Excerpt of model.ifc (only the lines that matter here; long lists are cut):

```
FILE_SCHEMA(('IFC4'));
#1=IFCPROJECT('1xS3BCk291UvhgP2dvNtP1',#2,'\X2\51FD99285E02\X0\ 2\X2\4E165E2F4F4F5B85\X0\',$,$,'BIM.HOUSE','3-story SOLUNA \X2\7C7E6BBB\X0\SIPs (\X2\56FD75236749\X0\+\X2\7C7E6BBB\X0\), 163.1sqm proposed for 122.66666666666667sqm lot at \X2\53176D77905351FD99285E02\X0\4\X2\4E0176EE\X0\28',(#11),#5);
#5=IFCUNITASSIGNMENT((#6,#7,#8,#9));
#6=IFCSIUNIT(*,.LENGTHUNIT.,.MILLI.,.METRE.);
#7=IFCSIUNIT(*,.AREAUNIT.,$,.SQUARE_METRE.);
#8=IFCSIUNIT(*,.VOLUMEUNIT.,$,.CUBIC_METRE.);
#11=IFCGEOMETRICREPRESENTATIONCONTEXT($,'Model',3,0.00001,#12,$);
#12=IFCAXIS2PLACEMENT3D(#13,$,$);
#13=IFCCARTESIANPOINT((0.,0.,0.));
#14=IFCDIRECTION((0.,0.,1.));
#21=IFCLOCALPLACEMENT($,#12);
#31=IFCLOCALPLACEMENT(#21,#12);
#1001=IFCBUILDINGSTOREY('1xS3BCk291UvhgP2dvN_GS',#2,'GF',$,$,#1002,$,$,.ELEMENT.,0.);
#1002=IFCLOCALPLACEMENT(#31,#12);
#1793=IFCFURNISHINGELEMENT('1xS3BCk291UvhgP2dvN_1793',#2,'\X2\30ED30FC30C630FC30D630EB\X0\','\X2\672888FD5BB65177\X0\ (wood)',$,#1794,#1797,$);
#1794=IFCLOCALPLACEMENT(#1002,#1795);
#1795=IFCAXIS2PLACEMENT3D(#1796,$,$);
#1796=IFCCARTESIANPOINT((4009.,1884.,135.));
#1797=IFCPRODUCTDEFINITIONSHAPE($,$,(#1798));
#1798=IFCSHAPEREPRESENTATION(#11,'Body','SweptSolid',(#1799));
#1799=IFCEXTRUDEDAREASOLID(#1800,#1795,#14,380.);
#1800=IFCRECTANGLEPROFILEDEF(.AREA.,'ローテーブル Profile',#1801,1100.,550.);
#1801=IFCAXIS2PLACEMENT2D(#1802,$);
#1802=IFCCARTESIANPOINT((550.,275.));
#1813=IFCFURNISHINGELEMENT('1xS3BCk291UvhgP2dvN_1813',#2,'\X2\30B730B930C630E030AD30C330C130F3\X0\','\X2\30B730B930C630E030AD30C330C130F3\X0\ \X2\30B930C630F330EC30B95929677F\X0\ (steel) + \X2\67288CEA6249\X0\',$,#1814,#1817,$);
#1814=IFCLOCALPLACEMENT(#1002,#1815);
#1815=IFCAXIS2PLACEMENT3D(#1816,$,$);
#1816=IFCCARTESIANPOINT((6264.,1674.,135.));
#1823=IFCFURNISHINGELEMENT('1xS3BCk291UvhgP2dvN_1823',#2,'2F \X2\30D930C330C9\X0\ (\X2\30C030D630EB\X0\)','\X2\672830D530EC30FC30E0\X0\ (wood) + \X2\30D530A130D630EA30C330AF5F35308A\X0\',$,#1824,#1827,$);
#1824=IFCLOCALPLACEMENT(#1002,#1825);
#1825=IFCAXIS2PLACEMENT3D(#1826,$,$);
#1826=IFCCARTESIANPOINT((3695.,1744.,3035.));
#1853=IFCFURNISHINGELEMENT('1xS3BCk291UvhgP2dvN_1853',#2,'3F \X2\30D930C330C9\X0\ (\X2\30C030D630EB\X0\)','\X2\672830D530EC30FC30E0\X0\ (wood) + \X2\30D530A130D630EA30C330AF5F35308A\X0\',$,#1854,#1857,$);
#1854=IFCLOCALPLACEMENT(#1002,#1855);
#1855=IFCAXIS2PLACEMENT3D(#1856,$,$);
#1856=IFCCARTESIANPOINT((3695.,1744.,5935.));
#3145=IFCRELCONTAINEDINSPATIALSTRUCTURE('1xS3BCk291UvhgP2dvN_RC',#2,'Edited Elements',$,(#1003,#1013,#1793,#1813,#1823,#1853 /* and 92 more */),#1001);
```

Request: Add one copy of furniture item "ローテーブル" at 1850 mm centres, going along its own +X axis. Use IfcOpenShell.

```python
import ifcopenshell
import ifcopenshell.api.geometry
import ifcopenshell.api.root
import ifcopenshell.util.element
import ifcopenshell.util.placement

model = ifcopenshell.open("model.ifc")


def reuse_history(source, copy):
    """copy_class also copies each property set's owner history, people and application; keep the originals."""
    for rel in copy.IsDefinedBy:
        if rel.is_a("IfcRelDefinesByProperties") and (history := rel.RelatingPropertyDefinition.OwnerHistory):
            rel.RelatingPropertyDefinition.OwnerHistory = source.OwnerHistory
            ifcopenshell.util.element.remove_deep2(model, history)


source = model.by_guid("1xS3BCk291UvhgP2dvN_1793")
base = ifcopenshell.util.placement.get_local_placement(source.ObjectPlacement)
step = base[:3, 0] * 1850.0

for i in range(1, 2):
    copy = ifcopenshell.api.root.copy_class(model, product=source)
    copy.Representation = ifcopenshell.util.element.copy_deep(
        model, source.Representation, exclude=["IfcGeometricRepresentationContext", "IfcRepresentationMap"]
    )
    reuse_history(source, copy)
    matrix = base.copy()
    matrix[:3, 3] += i * step
    print("added at", matrix[:3, 3].round(3) + 0.0)
    ifcopenshell.api.geometry.edit_object_placement(model, product=copy, matrix=matrix, is_si=False)

model.write("model_v2.ifc")
```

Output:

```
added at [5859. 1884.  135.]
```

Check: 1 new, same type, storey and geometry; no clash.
